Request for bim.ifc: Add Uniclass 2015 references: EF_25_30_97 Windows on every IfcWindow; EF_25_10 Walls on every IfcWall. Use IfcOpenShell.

First a look at what the model holds.

```python
import ifcopenshell

model = ifcopenshell.open("bim.ifc")
print(model.schema)
print("classifications:", [c.Name for c in model.by_type("IfcClassification")])
for ifc_class in ("IfcDoor", "IfcRoof", "IfcStair", "IfcWall", "IfcWindow"):
    print(ifc_class, len(model.by_type(ifc_class)))
```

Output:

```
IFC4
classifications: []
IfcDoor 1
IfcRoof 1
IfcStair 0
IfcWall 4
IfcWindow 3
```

```python
import ifcopenshell
import ifcopenshell.api.classification

model = ifcopenshell.open("bim.ifc")

system = ifcopenshell.api.classification.add_classification(model, classification="Uniclass 2015")

codes = {
    "IfcWindow": ("EF_25_30_97", "Windows"),
    "IfcWall": ("EF_25_10", "Walls"),
}
for ifc_class, (code, name) in codes.items():
    products = model.by_type(ifc_class)
    ifcopenshell.api.classification.add_reference(
        model, products=products, classification=system, identification=code, name=name
    )
    print(code, len(products))

model.write("bim_edited.ifc")
```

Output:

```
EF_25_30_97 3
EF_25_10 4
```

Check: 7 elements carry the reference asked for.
